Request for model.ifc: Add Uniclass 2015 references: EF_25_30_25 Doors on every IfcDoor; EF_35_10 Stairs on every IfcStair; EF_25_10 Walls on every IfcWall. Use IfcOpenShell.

First a look at what the model holds.

```python
import ifcopenshell

model = ifcopenshell.open("model.ifc")
print(model.schema)
print("classifications:", [c.Name for c in model.by_type("IfcClassification")])
for ifc_class in ("IfcDoor", "IfcRoof", "IfcStair", "IfcWall", "IfcWindow"):
    print(ifc_class, len(model.by_type(ifc_class)))
```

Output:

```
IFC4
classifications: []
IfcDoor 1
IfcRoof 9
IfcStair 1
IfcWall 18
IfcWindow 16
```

```python
import ifcopenshell
import ifcopenshell.api.classification

model = ifcopenshell.open("model.ifc")

system = ifcopenshell.api.classification.add_classification(model, classification="Uniclass 2015")

codes = {
    "IfcDoor": ("EF_25_30_25", "Doors"),
    "IfcStair": ("EF_35_10", "Stairs"),
    "IfcWall": ("EF_25_10", "Walls"),
}
for ifc_class, (code, name) in codes.items():
    products = model.by_type(ifc_class)
    ifcopenshell.api.classification.add_reference(
        model, products=products, classification=system, identification=code, name=name
    )
    print(code, len(products))

model.write("model_updated.ifc")
```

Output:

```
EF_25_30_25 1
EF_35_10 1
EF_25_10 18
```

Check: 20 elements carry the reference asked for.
